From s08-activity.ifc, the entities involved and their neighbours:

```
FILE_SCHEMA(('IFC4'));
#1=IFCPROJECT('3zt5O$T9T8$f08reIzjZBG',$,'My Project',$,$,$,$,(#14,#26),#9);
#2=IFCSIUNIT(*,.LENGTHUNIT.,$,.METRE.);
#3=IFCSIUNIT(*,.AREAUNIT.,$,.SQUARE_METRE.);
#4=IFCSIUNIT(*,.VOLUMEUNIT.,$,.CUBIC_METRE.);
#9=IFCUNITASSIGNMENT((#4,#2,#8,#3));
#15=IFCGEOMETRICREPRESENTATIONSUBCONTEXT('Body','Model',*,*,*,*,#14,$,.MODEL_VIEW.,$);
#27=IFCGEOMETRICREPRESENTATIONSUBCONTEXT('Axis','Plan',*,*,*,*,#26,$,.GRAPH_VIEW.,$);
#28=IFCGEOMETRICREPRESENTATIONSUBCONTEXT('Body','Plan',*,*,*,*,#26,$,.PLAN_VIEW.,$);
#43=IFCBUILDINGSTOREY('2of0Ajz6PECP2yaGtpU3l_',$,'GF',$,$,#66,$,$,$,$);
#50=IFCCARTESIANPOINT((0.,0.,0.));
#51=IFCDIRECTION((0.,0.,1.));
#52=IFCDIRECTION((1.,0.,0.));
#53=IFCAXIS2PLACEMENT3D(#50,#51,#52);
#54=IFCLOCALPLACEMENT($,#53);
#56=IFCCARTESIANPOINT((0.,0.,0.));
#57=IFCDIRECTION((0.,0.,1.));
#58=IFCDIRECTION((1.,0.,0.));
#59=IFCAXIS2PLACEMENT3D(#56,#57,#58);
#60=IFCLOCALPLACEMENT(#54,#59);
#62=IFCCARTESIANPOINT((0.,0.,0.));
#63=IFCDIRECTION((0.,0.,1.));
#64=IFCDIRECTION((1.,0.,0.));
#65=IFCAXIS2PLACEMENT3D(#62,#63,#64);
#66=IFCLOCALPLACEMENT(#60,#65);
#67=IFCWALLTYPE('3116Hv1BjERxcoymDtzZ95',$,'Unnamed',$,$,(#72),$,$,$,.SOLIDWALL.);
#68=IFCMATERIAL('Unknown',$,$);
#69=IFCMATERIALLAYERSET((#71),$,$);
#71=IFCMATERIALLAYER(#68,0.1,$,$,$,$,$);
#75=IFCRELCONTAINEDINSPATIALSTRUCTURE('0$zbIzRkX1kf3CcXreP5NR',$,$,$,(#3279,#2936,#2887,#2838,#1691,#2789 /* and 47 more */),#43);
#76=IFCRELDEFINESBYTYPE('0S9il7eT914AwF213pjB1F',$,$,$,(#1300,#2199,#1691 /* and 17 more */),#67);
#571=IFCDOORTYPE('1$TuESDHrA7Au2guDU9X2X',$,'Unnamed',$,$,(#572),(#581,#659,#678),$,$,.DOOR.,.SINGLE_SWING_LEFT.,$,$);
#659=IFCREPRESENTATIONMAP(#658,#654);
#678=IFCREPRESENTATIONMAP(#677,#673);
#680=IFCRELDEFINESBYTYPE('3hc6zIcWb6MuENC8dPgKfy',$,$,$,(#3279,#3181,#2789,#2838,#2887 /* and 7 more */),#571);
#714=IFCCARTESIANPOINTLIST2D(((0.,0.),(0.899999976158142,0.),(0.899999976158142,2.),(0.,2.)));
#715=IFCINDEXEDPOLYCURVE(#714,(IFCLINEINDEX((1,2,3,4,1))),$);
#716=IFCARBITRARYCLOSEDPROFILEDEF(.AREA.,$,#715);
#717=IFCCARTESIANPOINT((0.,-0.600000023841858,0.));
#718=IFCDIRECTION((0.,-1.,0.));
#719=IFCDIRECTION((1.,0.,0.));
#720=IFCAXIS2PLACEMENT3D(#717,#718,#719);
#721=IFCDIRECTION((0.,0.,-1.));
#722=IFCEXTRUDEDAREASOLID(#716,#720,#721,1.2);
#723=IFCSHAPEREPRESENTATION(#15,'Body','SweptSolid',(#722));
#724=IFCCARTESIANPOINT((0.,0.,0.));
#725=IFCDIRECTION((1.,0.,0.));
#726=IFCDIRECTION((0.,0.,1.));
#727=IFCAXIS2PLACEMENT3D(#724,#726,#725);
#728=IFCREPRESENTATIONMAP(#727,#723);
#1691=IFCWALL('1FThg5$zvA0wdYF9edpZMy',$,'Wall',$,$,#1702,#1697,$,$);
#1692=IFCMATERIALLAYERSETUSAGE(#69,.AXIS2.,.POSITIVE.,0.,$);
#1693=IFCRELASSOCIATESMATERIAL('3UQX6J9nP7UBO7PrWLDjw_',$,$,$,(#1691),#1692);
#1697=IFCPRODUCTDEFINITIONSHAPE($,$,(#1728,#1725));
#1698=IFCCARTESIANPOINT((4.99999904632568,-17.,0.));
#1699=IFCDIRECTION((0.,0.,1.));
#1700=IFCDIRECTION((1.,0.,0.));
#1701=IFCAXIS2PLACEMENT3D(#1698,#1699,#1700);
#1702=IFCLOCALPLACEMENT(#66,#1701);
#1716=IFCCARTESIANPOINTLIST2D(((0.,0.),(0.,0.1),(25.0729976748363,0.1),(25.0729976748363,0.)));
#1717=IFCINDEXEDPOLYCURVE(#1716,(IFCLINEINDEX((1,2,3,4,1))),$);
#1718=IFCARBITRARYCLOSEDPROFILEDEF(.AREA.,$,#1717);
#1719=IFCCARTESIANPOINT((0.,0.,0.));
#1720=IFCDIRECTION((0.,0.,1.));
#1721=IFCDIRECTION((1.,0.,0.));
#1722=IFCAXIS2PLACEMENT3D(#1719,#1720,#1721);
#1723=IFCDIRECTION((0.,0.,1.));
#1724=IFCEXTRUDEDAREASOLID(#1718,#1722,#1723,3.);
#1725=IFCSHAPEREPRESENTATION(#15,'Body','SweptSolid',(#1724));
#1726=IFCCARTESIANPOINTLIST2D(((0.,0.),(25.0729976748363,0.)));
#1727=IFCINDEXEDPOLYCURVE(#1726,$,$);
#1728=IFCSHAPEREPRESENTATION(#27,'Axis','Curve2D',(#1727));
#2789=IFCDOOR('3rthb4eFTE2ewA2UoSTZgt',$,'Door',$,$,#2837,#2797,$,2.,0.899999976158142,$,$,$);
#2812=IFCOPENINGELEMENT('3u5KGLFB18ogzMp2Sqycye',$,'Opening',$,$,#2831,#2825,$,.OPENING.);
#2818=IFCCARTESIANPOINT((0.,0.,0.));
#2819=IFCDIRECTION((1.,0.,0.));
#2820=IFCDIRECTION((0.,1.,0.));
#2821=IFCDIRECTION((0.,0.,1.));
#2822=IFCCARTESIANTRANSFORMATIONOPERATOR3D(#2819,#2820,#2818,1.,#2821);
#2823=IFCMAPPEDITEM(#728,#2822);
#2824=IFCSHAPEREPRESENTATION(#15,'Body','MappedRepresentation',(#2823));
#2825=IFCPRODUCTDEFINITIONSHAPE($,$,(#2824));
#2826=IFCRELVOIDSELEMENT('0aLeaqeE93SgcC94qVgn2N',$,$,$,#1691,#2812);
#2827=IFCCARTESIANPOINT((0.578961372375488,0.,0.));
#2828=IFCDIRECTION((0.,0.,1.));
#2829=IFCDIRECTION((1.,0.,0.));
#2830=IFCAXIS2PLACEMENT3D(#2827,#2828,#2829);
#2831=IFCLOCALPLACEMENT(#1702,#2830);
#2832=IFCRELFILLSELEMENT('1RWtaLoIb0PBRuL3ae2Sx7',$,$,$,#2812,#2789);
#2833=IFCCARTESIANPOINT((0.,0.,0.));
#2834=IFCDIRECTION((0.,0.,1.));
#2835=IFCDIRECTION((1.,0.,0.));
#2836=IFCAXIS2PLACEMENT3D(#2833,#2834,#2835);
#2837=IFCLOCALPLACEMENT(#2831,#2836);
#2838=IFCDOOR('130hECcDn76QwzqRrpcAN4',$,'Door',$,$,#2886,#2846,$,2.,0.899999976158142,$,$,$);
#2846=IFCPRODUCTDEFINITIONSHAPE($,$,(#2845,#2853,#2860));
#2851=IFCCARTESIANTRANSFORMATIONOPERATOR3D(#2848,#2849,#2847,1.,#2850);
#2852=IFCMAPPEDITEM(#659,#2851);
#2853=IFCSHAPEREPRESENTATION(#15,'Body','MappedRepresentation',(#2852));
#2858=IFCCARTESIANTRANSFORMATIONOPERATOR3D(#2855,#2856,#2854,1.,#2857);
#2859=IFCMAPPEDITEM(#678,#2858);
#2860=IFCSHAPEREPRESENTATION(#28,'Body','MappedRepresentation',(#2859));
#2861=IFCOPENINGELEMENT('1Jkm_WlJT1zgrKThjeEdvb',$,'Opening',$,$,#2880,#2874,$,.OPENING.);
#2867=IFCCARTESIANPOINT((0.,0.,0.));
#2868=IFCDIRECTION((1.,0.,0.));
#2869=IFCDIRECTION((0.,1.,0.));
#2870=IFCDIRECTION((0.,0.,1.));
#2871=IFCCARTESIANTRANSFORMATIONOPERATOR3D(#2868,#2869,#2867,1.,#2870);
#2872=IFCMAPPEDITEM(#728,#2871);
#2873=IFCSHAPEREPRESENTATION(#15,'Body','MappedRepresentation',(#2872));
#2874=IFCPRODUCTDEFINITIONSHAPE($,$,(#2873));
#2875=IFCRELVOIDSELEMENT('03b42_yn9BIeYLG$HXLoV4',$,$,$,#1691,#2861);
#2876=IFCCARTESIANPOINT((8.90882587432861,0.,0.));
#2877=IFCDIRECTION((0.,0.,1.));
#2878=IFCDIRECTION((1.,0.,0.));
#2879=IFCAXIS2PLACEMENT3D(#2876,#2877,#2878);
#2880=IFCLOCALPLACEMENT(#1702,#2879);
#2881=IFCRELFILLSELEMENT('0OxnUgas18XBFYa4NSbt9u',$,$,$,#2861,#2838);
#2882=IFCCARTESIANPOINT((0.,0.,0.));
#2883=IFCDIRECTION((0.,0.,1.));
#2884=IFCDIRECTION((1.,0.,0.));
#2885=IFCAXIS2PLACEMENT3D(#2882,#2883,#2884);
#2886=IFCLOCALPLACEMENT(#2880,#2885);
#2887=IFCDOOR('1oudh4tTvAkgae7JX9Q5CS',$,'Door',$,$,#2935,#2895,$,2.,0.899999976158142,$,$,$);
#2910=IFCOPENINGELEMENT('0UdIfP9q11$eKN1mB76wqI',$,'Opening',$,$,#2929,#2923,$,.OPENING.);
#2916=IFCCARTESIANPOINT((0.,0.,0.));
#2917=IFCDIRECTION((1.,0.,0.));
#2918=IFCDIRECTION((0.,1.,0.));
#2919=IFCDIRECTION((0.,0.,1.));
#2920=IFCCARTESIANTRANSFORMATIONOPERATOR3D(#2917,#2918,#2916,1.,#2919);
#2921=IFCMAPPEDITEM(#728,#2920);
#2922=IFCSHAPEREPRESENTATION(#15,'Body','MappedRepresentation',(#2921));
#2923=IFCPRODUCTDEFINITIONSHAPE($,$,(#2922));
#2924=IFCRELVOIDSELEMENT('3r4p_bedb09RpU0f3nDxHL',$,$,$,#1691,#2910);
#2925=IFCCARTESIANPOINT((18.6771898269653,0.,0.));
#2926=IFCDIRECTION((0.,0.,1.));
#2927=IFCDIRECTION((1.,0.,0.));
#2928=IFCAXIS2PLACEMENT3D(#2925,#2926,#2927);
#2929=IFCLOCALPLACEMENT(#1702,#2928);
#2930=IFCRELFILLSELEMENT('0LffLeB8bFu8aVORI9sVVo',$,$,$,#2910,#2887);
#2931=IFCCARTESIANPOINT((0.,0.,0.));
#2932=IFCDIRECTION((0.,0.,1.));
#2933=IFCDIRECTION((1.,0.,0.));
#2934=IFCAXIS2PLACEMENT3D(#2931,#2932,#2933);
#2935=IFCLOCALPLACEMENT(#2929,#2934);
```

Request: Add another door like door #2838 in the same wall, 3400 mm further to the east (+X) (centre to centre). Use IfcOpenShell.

```python
import ifcopenshell
import ifcopenshell.api.feature
import ifcopenshell.api.geometry
import ifcopenshell.api.root
import ifcopenshell.geom
import ifcopenshell.util.element
import ifcopenshell.util.placement
import ifcopenshell.util.shape
import ifcopenshell.util.unit

model = ifcopenshell.open("s08-activity.ifc")
unit_scale = ifcopenshell.util.unit.calculate_unit_scale(model)
settings = ifcopenshell.geom.settings()


def volume(element):
    """Net volume in cubic metres, openings subtracted."""
    shape = ifcopenshell.geom.create_shape(settings, element)
    return ifcopenshell.util.shape.get_volume(shape.geometry)


door = model.by_guid("130hECcDn76QwzqRrpcAN4")
opening = door.FillsVoids[0].RelatingOpeningElement
wall = opening.VoidsElements[0].RelatingBuildingElement
before = volume(wall)
shift = ifcopenshell.util.placement.get_local_placement(wall.ObjectPlacement)[:3, 0] * 3.4 / unit_scale

# copy_class copies the void relationship, type, container and properties, but no geometry.
new_opening = ifcopenshell.api.root.copy_class(model, product=opening)
new_opening.Representation = ifcopenshell.util.element.copy_deep(
    model, opening.Representation, exclude=["IfcGeometricRepresentationContext", "IfcRepresentationMap"]
)
new_door = ifcopenshell.api.root.copy_class(model, product=door)
new_door.Representation = ifcopenshell.util.element.copy_deep(
    model, door.Representation, exclude=["IfcGeometricRepresentationContext", "IfcRepresentationMap"]
)
ifcopenshell.api.feature.add_filling(model, opening=new_opening, element=new_door)

for old, new in ((opening, new_opening), (door, new_door)):
    matrix = ifcopenshell.util.placement.get_local_placement(old.ObjectPlacement)
    matrix[:3, 3] += shift
    ifcopenshell.api.geometry.edit_object_placement(model, product=new, matrix=matrix, is_si=False)

after = volume(wall)

print(f"wall volume {before:.3f} -> {after:.3f} m3")

model.write("s08-activity_updated.ifc")
```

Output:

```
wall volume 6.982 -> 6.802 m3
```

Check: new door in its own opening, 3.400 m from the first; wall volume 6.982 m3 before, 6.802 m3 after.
